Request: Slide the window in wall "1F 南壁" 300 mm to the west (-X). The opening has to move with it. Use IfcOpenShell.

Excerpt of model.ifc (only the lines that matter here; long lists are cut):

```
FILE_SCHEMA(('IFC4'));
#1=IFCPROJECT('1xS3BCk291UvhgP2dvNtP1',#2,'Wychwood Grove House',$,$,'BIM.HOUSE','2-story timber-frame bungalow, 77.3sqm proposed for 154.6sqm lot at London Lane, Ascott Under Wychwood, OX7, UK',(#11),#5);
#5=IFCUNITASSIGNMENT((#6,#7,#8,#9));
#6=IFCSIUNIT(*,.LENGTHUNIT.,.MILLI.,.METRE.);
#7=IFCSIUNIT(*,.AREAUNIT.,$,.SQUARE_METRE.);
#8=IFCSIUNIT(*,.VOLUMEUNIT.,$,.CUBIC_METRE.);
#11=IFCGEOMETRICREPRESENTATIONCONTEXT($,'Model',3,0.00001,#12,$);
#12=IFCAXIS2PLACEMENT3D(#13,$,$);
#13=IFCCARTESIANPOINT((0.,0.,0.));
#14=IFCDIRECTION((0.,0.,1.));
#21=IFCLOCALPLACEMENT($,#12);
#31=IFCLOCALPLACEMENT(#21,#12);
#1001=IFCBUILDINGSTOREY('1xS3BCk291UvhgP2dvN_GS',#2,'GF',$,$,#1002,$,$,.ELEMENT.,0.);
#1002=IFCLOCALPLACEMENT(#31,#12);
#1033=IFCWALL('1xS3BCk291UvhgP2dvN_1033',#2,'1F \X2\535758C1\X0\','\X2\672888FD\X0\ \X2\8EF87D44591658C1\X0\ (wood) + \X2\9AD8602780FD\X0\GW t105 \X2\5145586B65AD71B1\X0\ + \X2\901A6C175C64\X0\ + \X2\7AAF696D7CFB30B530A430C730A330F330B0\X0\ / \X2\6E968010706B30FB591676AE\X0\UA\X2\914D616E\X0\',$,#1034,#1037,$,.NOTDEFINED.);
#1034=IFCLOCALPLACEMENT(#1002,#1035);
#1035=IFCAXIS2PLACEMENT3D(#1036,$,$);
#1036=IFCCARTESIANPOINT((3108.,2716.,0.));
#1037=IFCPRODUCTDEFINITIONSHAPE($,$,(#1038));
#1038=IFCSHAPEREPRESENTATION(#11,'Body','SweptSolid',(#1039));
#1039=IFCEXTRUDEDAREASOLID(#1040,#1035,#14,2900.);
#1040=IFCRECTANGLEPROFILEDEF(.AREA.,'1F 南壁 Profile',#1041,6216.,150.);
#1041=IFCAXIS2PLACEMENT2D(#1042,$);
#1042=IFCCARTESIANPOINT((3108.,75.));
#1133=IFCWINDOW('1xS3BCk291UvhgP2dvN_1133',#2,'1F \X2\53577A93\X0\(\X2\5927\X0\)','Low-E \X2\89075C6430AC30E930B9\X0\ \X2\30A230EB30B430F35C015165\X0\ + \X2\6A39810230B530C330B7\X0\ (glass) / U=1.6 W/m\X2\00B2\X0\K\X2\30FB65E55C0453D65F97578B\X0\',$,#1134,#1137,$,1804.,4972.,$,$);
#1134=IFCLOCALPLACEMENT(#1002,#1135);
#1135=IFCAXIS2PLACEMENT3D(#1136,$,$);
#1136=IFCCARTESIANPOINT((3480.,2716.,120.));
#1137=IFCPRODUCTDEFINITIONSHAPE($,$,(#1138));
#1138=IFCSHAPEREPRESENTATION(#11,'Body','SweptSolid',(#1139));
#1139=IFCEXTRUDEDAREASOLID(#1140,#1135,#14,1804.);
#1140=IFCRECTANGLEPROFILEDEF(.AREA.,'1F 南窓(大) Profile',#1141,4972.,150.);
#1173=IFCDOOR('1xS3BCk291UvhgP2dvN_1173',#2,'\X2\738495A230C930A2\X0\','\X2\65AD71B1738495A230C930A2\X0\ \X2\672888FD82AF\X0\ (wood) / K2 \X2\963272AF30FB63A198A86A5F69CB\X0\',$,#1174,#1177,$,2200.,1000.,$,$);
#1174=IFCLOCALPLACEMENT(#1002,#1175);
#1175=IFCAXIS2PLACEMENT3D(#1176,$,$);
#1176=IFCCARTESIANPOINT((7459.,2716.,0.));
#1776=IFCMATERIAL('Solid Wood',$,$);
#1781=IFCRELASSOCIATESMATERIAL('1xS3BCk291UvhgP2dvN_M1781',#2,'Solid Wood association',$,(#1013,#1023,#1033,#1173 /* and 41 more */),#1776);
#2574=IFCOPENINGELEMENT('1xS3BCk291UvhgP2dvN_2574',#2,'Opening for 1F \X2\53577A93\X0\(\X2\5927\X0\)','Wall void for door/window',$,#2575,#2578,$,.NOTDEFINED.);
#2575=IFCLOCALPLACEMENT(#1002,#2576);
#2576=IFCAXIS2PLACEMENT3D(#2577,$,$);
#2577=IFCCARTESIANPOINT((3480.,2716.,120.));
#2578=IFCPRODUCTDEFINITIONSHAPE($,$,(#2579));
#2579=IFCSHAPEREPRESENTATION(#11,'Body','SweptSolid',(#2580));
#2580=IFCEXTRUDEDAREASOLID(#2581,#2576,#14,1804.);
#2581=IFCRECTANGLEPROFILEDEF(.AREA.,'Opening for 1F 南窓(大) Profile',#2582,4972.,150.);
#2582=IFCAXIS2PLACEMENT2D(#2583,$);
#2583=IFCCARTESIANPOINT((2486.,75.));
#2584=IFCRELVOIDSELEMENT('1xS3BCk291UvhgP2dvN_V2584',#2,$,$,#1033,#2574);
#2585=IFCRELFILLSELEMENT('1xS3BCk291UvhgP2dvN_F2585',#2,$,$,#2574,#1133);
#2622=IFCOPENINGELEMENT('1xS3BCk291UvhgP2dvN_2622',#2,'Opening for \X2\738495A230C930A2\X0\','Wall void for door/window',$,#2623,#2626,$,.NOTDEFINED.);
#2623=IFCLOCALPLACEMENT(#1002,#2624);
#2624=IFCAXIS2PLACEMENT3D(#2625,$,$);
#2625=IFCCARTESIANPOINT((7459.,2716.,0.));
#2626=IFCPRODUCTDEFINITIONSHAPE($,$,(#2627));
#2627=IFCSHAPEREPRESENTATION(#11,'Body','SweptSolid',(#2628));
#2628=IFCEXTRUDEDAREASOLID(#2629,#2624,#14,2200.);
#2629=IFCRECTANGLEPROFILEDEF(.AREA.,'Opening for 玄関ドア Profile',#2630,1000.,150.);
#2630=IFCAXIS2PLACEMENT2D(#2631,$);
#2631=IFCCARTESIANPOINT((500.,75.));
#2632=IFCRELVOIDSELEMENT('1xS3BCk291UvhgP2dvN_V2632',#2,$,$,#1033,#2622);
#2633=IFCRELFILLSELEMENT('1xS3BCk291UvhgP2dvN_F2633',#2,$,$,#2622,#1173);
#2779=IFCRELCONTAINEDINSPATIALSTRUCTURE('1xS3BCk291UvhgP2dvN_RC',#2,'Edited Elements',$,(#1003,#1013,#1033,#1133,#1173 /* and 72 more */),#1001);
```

```python
import ifcopenshell
import ifcopenshell.api.geometry
import ifcopenshell.util.placement

model = ifcopenshell.open("model.ifc")

window = model.by_guid("1xS3BCk291UvhgP2dvN_1133")
opening = window.FillsVoids[0].RelatingOpeningElement
wall = opening.VoidsElements[0].RelatingBuildingElement

wall_matrix = ifcopenshell.util.placement.get_local_placement(wall.ObjectPlacement)
shift = wall_matrix[:3, 0] * -300.0
before = ifcopenshell.util.placement.get_local_placement(window.ObjectPlacement)[:3, 3].copy()

# The window is not placed relative to its opening, so move both.
for product in (opening, window):
    matrix = ifcopenshell.util.placement.get_local_placement(product.ObjectPlacement)
    matrix[:3, 3] += shift
    ifcopenshell.api.geometry.edit_object_placement(model, product=product, matrix=matrix, is_si=False)

after = ifcopenshell.util.placement.get_local_placement(window.ObjectPlacement)[:3, 3]
print("window moved by", (after - before).round(3) + 0.0)

model.write("model_v2.ifc")
```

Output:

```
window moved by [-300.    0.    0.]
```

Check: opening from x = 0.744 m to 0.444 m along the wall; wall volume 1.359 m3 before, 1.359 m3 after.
